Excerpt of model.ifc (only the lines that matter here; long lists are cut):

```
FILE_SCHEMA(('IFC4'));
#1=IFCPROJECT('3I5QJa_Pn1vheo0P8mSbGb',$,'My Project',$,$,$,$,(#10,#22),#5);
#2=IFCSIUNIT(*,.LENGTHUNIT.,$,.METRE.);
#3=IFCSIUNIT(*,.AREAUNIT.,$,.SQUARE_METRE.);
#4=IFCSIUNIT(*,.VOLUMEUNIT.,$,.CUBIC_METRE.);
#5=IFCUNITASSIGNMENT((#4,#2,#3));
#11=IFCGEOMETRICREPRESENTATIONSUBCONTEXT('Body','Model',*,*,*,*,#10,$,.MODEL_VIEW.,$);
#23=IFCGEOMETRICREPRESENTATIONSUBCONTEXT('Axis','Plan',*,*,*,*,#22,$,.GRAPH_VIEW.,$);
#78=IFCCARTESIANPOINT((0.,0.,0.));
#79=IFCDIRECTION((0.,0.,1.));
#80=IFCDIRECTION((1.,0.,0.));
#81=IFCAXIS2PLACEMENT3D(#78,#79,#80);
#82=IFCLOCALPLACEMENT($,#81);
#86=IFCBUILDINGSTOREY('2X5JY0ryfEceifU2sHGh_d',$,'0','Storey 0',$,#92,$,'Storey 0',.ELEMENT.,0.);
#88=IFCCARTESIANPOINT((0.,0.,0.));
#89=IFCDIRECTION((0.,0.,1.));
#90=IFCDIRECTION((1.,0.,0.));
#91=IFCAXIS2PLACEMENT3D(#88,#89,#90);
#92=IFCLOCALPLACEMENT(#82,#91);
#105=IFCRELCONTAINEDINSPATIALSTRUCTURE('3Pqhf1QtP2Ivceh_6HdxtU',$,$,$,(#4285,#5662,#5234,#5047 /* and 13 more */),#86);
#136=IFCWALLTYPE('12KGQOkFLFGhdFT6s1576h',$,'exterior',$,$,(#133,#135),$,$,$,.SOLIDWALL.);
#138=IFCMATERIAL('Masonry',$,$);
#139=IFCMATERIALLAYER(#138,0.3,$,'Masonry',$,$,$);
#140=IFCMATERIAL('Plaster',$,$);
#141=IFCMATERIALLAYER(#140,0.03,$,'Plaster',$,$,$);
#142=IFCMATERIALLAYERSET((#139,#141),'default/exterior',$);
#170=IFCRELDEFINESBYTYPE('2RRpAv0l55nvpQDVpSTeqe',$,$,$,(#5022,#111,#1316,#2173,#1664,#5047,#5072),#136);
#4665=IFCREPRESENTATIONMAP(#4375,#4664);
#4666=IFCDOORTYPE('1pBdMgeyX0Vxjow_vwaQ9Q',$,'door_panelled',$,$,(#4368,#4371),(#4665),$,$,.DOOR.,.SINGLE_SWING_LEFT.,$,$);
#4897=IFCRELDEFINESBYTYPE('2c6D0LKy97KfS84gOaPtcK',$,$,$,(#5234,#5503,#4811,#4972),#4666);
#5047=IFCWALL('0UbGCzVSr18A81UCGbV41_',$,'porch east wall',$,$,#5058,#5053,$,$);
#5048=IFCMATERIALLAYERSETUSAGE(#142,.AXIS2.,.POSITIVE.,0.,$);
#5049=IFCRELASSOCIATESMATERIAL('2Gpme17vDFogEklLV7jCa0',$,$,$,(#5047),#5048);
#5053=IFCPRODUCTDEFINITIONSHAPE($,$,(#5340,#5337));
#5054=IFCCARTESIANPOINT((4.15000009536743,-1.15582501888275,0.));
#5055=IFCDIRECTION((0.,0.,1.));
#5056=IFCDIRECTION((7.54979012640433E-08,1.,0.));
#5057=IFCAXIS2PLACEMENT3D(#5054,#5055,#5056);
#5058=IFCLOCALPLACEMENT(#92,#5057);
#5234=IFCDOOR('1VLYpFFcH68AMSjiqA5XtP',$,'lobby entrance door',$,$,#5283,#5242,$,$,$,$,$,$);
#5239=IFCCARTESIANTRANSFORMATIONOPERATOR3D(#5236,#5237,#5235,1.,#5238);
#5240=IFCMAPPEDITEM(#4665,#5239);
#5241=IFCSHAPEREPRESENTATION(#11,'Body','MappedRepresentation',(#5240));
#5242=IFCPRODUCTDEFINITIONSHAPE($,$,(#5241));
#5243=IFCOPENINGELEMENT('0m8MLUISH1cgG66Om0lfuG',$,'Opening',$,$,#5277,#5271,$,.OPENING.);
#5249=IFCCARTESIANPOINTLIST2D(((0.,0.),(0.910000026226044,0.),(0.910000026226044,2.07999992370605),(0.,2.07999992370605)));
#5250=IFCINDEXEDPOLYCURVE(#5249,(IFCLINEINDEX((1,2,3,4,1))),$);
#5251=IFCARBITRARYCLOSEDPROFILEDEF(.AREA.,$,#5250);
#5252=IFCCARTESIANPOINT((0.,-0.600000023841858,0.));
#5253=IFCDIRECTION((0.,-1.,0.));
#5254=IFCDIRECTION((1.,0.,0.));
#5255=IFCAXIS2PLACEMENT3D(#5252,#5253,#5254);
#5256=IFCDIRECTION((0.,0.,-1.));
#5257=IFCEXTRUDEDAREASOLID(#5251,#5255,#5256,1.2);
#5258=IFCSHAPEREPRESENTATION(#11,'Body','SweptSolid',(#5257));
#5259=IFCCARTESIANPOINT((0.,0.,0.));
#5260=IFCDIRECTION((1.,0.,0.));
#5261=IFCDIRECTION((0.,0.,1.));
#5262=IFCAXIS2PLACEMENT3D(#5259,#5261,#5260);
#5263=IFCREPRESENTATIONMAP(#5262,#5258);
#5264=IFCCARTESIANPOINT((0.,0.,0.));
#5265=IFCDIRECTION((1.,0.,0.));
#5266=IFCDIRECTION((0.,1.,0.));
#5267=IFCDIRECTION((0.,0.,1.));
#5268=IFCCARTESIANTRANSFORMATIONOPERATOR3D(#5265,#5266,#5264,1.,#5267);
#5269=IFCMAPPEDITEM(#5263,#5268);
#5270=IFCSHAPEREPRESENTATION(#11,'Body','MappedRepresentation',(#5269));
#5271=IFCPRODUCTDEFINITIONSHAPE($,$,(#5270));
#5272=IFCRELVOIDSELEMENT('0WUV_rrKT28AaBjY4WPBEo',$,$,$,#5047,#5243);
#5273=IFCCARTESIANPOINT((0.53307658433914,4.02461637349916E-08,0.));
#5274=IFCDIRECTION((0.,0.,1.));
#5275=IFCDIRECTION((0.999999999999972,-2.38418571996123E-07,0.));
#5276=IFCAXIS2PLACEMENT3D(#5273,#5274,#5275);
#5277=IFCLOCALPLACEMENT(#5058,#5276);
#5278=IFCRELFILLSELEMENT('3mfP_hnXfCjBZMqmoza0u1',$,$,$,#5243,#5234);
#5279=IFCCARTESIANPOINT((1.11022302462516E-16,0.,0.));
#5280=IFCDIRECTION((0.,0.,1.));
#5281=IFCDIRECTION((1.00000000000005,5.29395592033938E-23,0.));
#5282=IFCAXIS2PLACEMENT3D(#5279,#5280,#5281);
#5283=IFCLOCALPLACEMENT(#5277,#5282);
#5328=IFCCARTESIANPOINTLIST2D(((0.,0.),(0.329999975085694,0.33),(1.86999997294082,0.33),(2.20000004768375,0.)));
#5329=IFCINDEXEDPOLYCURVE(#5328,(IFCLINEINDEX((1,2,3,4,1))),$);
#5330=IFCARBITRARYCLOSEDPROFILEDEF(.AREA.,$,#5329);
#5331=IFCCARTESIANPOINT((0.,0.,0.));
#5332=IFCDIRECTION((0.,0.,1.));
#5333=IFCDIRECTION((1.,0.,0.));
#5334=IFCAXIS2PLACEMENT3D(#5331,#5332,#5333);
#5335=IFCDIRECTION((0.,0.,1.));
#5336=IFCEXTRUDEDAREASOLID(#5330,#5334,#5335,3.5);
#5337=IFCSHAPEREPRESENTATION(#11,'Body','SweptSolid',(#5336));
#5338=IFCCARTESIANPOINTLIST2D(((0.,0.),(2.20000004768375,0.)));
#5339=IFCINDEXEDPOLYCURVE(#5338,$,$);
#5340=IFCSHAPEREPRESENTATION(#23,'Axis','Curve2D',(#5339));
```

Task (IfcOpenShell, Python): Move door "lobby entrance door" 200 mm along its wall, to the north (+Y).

```python
import ifcopenshell
import ifcopenshell.api.geometry
import ifcopenshell.util.placement
import ifcopenshell.util.unit

model = ifcopenshell.open("model.ifc")
unit_scale = ifcopenshell.util.unit.calculate_unit_scale(model)

door = model.by_id(5234)
opening = door.FillsVoids[0].RelatingOpeningElement
wall = opening.VoidsElements[0].RelatingBuildingElement

wall_matrix = ifcopenshell.util.placement.get_local_placement(wall.ObjectPlacement)
shift = wall_matrix[:3, 0] * 0.2 / unit_scale
before = ifcopenshell.util.placement.get_local_placement(door.ObjectPlacement)[:3, 3].copy()

# The door is placed relative to its opening, so it follows when the opening moves.
matrix = ifcopenshell.util.placement.get_local_placement(opening.ObjectPlacement)
matrix[:3, 3] += shift
ifcopenshell.api.geometry.edit_object_placement(
    model, product=opening, matrix=matrix, is_si=False, should_transform_children=True
)

after = ifcopenshell.util.placement.get_local_placement(door.ObjectPlacement)[:3, 3]
print("door moved by", (after - before).round(3) + 0.0)

model.write("model_updated.ifc")
```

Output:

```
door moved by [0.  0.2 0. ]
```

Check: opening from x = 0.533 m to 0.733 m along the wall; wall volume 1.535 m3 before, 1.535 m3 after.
